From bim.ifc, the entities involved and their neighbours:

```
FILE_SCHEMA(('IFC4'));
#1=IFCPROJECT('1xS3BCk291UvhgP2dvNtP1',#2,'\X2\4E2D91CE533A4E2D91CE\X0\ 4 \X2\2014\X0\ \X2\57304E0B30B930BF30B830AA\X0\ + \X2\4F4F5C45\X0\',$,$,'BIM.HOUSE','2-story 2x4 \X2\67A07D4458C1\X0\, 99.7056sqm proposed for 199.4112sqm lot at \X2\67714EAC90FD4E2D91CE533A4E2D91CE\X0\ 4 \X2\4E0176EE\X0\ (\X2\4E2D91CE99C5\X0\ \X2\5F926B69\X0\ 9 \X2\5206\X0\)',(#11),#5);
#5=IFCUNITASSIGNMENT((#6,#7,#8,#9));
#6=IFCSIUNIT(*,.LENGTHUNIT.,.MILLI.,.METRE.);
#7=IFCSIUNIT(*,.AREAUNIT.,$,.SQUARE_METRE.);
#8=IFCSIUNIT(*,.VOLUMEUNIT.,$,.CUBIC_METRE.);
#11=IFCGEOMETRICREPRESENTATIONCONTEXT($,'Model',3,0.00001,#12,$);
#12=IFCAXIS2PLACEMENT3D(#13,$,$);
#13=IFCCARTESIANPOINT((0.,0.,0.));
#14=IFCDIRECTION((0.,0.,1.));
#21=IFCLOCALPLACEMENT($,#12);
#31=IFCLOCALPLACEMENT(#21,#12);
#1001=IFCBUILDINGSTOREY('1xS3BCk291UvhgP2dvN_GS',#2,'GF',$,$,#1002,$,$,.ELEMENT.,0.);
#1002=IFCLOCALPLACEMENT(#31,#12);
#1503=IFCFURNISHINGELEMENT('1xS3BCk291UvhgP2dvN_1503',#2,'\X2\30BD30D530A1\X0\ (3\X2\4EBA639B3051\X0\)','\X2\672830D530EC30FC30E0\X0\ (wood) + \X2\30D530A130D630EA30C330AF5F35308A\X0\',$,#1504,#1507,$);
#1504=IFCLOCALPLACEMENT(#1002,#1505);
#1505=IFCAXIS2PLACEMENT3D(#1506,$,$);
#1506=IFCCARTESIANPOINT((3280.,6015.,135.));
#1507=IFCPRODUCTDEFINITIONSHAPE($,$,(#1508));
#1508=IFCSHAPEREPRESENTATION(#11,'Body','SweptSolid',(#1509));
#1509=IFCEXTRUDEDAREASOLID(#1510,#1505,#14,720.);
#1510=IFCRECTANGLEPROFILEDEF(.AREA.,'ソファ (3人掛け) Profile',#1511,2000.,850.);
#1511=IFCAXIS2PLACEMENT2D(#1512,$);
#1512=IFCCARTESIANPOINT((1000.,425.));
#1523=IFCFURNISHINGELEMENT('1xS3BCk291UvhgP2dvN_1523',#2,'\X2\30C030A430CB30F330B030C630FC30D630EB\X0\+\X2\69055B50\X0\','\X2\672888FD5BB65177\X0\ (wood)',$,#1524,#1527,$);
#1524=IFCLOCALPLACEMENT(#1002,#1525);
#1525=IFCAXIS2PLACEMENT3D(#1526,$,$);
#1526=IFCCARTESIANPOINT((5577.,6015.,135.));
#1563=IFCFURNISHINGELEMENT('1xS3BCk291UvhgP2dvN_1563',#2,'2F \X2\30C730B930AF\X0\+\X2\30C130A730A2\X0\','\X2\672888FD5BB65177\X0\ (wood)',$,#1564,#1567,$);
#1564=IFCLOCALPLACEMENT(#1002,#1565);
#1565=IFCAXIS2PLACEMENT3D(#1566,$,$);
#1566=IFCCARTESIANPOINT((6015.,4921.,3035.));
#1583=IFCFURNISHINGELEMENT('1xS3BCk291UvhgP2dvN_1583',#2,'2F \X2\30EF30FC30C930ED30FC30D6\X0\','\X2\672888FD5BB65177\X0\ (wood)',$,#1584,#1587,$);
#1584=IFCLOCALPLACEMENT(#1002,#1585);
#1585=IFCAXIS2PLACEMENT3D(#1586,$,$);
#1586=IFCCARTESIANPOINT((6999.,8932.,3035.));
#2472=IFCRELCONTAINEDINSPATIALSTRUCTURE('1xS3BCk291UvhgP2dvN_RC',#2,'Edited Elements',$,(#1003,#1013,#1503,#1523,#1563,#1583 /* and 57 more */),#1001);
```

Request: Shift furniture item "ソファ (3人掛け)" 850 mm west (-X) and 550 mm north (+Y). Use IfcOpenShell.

```python
import ifcopenshell
import ifcopenshell.api.geometry
import ifcopenshell.util.placement

model = ifcopenshell.open("bim.ifc")

item = model.by_guid("1xS3BCk291UvhgP2dvN_1503")
matrix = ifcopenshell.util.placement.get_local_placement(item.ObjectPlacement)
matrix[0, 3] -= 850.0
matrix[1, 3] += 550.0
ifcopenshell.api.geometry.edit_object_placement(model, product=item, matrix=matrix, is_si=False)

print(ifcopenshell.util.placement.get_local_placement(item.ObjectPlacement).round(3) + 0.0)

model.write("bim_v2.ifc")
```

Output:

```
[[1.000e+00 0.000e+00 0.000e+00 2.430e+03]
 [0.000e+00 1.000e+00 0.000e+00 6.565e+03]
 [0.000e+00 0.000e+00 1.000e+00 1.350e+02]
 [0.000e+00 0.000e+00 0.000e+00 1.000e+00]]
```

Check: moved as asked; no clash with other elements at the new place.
